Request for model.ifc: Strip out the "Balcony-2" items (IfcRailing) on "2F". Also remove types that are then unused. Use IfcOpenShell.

First a look at what the model holds.

```python
import ifcopenshell
import ifcopenshell.util.element

model = ifcopenshell.open("model.ifc")
print(model.schema)
storey = next(s for s in model.by_type("IfcBuildingStorey") if s.Name == "2F")
railings = [e for e in ifcopenshell.util.element.get_decomposition(storey) if e.is_a("IfcRailing")]
seen = {}
for e in railings:
    element_type = ifcopenshell.util.element.get_type(e)
    name = element_type.Name if element_type not in (None, e) else None
    seen[name] = seen.get(name, 0) + 1
for name, count in sorted(seen.items(), key=str):
    print(count, "x", name)
```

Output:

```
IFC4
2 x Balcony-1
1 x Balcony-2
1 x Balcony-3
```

```python
import ifcopenshell
import ifcopenshell.api.root
import ifcopenshell.util.element

model = ifcopenshell.open("model.ifc")

storey = next(s for s in model.by_type("IfcBuildingStorey") if s.Name == "2F")
railings = [e for e in ifcopenshell.util.element.get_decomposition(storey) if e.is_a("IfcRailing")]
targets = [e for e in railings if (t := ifcopenshell.util.element.get_type(e)) not in (None, e) and t.Name == "Balcony-2"]
types = {ifcopenshell.util.element.get_type(e) for e in targets} - {None, *targets}

for e in targets:
    ifcopenshell.api.root.remove_product(model, product=e)
print(len(targets), "removed")

unused = [t for t in types if not ifcopenshell.util.element.get_types(t)]
for t in unused:
    ifcopenshell.api.root.remove_product(model, product=t)
print(len(unused), "unused types removed")

model.write("model_updated.ifc")
```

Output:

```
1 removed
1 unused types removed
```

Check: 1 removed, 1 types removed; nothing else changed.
